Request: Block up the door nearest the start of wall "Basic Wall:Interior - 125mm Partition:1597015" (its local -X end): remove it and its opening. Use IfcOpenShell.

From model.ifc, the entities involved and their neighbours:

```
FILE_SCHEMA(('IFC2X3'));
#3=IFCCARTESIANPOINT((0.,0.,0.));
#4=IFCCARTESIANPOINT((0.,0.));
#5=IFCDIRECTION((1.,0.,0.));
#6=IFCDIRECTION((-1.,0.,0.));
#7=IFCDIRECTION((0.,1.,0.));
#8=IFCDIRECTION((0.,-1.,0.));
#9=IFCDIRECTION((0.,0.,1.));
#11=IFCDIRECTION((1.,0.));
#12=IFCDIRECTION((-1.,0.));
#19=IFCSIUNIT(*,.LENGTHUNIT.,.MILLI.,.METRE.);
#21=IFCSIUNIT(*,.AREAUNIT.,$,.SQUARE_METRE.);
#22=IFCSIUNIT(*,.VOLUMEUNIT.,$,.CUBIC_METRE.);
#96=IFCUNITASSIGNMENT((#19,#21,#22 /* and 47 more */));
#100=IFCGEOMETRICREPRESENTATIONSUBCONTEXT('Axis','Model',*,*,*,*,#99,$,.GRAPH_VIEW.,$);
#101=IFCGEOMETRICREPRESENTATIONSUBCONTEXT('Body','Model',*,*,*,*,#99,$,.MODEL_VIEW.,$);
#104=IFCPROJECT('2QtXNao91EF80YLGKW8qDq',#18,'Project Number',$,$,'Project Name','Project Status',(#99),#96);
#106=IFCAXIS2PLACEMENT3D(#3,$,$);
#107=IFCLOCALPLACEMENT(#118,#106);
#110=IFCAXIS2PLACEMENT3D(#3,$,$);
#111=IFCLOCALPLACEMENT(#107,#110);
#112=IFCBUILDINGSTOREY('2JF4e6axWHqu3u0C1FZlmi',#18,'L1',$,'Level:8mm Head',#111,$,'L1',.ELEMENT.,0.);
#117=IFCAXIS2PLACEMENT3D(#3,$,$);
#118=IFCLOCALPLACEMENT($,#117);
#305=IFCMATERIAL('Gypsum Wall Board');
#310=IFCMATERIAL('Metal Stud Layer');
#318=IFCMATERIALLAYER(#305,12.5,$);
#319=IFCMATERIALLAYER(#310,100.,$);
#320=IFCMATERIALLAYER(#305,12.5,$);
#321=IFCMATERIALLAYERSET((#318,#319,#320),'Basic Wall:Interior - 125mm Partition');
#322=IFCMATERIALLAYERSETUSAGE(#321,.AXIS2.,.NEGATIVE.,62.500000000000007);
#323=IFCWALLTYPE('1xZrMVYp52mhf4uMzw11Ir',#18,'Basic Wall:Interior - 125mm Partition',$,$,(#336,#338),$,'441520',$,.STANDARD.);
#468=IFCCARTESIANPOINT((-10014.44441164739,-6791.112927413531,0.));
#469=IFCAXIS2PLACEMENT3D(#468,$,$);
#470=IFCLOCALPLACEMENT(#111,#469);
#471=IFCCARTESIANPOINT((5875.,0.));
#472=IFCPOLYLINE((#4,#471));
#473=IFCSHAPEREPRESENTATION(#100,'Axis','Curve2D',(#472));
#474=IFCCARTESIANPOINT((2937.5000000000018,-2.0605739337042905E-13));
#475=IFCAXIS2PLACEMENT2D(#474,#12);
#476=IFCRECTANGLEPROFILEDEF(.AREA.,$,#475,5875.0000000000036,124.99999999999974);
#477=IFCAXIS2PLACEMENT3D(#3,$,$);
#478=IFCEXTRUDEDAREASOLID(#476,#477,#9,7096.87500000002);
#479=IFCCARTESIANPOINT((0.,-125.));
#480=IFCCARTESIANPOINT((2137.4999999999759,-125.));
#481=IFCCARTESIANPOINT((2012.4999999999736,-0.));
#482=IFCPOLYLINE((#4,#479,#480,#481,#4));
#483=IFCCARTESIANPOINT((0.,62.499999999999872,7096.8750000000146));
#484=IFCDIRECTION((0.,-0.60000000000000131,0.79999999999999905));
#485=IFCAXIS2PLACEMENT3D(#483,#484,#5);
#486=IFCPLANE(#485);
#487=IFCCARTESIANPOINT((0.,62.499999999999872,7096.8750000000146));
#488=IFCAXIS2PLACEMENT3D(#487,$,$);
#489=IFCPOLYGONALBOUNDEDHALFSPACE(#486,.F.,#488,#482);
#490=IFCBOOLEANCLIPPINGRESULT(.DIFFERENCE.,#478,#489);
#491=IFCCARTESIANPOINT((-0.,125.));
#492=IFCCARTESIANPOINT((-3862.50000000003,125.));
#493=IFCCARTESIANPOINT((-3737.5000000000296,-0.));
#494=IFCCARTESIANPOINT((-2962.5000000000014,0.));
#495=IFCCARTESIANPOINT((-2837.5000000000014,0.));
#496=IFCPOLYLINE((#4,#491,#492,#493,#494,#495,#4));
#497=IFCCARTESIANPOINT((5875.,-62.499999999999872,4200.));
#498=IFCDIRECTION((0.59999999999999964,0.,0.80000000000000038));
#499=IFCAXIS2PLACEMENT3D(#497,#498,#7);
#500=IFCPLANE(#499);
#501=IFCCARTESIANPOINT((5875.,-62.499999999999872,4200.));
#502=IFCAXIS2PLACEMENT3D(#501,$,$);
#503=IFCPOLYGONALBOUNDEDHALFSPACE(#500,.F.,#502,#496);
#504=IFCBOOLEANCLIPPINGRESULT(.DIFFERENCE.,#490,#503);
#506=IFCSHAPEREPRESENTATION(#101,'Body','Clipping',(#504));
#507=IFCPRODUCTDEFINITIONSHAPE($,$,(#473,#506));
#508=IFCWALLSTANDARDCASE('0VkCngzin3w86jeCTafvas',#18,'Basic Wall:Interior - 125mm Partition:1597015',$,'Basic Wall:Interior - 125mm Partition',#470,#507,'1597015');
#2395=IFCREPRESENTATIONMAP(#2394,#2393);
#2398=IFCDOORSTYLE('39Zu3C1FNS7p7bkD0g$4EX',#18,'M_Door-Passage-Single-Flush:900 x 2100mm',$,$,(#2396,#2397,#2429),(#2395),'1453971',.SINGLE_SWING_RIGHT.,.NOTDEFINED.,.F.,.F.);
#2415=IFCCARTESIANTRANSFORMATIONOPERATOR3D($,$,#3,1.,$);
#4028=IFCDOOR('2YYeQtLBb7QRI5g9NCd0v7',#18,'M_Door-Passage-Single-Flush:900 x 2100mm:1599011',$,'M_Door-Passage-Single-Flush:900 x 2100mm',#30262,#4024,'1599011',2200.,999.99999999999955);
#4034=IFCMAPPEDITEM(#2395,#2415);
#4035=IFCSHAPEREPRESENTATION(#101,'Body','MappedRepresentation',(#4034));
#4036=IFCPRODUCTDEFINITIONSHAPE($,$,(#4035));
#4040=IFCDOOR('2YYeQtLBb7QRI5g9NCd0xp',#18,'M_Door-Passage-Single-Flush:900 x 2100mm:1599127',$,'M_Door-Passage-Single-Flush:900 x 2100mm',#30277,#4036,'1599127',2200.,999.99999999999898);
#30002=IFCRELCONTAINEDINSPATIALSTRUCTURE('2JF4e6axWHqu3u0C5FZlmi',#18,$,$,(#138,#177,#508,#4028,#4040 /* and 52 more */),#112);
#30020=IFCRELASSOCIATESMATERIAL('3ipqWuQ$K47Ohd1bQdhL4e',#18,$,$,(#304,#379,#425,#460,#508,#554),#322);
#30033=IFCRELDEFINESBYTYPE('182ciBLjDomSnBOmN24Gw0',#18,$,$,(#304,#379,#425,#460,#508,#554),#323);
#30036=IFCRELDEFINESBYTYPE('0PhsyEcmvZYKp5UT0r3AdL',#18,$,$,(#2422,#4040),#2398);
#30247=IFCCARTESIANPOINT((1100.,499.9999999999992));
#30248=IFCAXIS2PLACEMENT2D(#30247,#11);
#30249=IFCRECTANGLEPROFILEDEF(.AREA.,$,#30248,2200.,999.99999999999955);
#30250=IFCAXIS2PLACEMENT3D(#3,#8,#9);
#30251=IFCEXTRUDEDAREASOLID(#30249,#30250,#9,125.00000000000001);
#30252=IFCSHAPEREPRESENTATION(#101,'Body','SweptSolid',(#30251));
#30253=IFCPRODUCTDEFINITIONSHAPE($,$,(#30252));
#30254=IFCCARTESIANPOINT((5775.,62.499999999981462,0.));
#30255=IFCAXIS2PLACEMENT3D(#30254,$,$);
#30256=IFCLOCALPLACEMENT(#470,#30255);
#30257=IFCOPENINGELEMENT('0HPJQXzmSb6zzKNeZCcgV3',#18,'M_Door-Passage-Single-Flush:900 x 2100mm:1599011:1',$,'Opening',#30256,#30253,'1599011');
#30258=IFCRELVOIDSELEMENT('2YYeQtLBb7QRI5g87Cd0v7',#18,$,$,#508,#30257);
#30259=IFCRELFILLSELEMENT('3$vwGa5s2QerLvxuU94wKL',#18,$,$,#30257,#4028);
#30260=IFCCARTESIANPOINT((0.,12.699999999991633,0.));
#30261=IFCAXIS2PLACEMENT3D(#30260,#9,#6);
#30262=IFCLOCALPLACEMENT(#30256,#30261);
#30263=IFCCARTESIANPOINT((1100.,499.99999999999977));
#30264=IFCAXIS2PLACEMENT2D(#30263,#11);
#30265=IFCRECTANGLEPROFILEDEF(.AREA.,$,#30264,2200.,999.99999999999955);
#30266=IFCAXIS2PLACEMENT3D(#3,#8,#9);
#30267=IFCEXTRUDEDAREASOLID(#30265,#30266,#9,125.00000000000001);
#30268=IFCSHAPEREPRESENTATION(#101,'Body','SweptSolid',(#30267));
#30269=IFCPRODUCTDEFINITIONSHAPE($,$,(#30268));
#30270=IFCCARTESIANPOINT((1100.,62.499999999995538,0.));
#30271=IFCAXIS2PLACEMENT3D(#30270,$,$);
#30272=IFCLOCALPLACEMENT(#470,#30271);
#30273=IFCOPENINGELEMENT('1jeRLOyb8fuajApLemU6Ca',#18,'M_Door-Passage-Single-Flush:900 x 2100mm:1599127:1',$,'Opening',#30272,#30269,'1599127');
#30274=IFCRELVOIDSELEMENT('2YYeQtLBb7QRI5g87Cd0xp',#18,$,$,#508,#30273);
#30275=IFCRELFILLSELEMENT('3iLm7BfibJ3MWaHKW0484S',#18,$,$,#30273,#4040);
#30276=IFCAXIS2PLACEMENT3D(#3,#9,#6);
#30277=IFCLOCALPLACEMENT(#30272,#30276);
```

```python
import ifcopenshell
import ifcopenshell.api.feature
import ifcopenshell.api.root
import ifcopenshell.geom
import ifcopenshell.util.shape

model = ifcopenshell.open("model.ifc")
settings = ifcopenshell.geom.settings()


def volume(element):
    """Net volume in cubic metres, openings subtracted."""
    shape = ifcopenshell.geom.create_shape(settings, element)
    return ifcopenshell.util.shape.get_volume(shape.geometry)


door = model.by_guid("2YYeQtLBb7QRI5g9NCd0xp")
opening = door.FillsVoids[0].RelatingOpeningElement
wall = opening.VoidsElements[0].RelatingBuildingElement
before = volume(wall)

ifcopenshell.api.root.remove_product(model, product=door)
ifcopenshell.api.feature.remove_feature(model, feature=opening)

after = volume(wall)

print(f"wall volume {before:.3f} -> {after:.3f} m3")

model.write("model_edited.ifc")
```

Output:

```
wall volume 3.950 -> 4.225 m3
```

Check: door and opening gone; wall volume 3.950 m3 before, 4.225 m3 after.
